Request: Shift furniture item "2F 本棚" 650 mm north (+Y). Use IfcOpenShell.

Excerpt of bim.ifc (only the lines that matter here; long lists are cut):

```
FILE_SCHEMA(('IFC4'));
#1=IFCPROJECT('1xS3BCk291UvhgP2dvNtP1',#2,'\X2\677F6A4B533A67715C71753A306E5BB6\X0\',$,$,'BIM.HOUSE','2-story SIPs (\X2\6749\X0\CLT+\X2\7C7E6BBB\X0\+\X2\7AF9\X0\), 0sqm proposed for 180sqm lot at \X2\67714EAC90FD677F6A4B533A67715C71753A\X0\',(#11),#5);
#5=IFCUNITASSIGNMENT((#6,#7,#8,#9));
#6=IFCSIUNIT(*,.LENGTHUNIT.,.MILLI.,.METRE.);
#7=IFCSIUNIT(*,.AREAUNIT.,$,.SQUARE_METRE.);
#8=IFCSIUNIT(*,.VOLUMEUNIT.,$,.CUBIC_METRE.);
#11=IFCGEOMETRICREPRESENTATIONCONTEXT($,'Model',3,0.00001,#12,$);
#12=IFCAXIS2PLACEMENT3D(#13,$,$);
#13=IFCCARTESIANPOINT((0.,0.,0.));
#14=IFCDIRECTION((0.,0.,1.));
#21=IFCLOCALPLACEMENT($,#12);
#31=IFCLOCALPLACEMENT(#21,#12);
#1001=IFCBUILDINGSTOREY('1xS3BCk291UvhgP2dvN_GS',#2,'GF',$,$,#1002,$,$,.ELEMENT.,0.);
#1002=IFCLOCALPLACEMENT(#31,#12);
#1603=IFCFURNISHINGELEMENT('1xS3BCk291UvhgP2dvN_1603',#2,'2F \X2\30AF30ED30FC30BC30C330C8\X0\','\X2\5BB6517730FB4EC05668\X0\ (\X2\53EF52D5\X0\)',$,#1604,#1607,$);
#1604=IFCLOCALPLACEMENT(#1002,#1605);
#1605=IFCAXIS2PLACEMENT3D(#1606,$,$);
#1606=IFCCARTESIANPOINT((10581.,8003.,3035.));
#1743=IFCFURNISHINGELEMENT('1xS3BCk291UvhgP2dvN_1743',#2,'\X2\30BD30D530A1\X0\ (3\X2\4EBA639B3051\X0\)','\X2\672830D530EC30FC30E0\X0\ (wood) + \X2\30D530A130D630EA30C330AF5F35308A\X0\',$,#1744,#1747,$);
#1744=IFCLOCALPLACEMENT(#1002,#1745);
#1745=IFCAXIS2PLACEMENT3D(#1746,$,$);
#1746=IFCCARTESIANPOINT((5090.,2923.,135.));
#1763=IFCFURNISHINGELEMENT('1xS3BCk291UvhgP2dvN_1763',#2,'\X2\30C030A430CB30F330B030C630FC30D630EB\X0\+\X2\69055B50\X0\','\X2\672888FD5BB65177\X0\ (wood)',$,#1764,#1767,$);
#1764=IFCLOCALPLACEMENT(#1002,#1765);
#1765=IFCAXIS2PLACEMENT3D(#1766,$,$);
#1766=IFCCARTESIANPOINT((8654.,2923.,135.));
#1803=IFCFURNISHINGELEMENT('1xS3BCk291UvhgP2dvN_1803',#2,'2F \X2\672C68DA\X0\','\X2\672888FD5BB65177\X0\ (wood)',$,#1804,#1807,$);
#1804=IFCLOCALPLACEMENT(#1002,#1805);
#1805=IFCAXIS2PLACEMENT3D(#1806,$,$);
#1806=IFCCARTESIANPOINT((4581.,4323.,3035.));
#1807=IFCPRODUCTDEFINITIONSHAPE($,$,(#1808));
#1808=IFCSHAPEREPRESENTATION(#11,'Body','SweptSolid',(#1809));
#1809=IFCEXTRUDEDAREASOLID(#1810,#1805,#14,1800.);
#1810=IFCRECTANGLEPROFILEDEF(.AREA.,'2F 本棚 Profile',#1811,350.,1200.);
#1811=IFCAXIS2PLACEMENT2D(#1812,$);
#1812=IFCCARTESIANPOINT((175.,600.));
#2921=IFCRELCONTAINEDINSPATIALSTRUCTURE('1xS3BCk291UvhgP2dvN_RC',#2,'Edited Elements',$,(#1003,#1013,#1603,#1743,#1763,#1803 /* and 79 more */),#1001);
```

```python
import ifcopenshell
import ifcopenshell.api.geometry
import ifcopenshell.util.placement
import ifcopenshell.util.unit

model = ifcopenshell.open("bim.ifc")
unit_scale = ifcopenshell.util.unit.calculate_unit_scale(model)

item = model.by_guid("1xS3BCk291UvhgP2dvN_1803")
matrix = ifcopenshell.util.placement.get_local_placement(item.ObjectPlacement)
matrix[1, 3] += 0.65 / unit_scale
ifcopenshell.api.geometry.edit_object_placement(model, product=item, matrix=matrix, is_si=False)

print(ifcopenshell.util.placement.get_local_placement(item.ObjectPlacement).round(3) + 0.0)

model.write("bim_v2.ifc")
```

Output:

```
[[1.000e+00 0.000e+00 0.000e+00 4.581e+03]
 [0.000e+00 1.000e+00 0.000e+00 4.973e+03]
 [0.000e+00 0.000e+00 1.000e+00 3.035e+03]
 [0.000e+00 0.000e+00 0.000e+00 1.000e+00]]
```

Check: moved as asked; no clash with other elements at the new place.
